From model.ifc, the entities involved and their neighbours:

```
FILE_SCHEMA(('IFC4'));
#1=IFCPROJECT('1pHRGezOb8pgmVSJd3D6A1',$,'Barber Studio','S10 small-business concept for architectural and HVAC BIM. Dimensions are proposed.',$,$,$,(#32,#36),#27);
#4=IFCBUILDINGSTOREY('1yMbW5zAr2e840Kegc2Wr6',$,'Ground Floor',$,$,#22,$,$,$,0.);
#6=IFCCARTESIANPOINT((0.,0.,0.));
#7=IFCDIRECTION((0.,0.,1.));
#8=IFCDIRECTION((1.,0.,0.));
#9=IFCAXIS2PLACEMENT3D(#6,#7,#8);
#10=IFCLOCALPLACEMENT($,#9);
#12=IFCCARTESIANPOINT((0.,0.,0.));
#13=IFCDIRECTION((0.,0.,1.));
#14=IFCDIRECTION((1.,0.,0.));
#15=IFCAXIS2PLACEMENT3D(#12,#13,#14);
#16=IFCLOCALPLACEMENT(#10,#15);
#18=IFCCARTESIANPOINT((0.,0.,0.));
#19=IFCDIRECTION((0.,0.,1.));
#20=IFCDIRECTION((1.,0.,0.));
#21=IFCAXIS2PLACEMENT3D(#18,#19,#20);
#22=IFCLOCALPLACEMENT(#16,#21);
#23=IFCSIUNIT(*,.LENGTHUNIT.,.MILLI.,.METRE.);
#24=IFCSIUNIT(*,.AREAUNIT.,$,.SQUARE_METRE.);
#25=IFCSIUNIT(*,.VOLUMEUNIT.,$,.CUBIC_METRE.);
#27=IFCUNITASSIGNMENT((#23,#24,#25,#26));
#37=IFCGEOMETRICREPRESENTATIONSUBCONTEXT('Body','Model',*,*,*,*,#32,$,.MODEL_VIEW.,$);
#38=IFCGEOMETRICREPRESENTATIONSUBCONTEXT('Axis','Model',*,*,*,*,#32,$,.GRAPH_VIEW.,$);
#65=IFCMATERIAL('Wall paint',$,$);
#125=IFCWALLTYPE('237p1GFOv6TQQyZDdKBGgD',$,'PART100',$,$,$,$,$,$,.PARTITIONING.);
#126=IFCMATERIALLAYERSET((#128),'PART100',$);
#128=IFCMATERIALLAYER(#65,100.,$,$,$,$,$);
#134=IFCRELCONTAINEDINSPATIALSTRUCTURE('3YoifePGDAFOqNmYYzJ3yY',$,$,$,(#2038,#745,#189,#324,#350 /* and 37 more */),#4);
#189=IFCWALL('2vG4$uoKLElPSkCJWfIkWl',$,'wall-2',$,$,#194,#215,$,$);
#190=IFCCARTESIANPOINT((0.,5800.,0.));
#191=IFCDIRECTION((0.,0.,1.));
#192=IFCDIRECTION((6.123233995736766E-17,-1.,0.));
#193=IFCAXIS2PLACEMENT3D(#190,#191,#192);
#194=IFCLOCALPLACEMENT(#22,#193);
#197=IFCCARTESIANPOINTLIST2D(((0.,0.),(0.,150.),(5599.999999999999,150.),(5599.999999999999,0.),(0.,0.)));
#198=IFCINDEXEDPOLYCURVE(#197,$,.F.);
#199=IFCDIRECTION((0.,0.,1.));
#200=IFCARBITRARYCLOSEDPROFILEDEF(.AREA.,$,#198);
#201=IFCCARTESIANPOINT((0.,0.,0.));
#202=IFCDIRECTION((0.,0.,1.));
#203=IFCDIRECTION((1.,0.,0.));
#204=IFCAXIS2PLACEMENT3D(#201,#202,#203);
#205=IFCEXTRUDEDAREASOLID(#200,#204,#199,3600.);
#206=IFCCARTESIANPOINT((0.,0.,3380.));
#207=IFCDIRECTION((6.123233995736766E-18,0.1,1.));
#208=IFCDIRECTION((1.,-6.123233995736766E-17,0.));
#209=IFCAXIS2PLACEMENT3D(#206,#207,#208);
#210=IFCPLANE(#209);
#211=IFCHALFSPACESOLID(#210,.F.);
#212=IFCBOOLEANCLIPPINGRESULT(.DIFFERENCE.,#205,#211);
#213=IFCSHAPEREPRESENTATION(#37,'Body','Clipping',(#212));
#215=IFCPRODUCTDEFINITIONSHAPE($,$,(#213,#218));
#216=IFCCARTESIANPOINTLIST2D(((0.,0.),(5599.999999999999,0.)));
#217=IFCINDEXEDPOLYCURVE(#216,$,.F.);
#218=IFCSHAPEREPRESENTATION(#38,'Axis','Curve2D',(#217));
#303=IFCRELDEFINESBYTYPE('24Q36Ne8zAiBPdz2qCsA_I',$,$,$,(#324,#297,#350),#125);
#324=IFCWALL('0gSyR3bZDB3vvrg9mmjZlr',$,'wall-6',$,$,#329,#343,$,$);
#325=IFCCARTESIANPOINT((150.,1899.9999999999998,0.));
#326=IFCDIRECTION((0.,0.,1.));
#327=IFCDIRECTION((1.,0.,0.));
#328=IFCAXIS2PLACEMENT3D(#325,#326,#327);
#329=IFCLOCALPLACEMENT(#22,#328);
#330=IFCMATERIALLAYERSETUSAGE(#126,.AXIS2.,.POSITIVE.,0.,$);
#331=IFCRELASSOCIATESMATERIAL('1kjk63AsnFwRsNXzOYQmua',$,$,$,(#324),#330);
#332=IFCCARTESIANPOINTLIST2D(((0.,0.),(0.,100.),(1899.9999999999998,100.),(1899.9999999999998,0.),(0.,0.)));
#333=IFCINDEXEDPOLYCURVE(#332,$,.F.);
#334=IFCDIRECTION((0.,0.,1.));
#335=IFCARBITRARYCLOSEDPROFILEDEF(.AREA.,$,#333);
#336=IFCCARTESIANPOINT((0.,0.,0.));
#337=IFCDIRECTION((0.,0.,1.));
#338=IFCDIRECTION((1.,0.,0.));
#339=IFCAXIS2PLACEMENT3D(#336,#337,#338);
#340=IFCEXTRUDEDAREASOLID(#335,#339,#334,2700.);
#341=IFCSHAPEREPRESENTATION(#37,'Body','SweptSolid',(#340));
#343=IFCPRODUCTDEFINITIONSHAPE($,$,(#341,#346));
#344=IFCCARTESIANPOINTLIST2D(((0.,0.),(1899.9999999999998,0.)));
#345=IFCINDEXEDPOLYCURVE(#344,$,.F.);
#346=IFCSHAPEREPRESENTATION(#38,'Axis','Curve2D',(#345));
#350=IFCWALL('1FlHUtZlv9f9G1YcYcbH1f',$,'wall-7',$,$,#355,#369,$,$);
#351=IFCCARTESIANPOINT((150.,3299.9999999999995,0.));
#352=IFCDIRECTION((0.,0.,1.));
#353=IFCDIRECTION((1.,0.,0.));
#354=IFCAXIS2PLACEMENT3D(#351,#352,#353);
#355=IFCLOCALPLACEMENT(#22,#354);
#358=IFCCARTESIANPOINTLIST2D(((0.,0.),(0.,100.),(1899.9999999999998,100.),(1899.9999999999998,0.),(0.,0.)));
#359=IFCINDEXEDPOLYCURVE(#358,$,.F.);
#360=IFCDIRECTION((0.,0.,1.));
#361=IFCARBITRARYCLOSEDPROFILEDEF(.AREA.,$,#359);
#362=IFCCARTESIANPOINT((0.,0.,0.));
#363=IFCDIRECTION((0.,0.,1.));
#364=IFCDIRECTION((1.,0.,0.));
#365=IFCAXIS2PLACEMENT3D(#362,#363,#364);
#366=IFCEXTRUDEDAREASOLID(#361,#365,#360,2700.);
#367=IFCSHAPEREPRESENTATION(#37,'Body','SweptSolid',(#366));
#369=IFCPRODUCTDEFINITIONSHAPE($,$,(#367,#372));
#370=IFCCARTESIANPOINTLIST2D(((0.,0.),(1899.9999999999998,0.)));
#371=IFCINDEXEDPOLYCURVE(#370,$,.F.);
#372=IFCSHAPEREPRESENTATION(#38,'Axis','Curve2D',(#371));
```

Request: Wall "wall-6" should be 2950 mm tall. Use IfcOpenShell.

```python
import ifcopenshell
import ifcopenshell.geom
import ifcopenshell.util.representation
import ifcopenshell.util.shape

model = ifcopenshell.open("model.ifc")
settings = ifcopenshell.geom.settings()


def volume(element):
    """Net volume in cubic metres, openings subtracted."""
    shape = ifcopenshell.geom.create_shape(settings, element)
    return ifcopenshell.util.shape.get_volume(shape.geometry)


wall = model.by_id(324)
before = volume(wall)

body = ifcopenshell.util.representation.get_representation(wall, "Model", "Body")
solid = body.Items[0]
old_height = solid.Depth
solid.Depth = 2950.0
after = volume(wall)

print(f"height {old_height:g} -> {solid.Depth:g}, volume {before:.3f} -> {after:.3f} m3")

model.write("model_updated.ifc")
```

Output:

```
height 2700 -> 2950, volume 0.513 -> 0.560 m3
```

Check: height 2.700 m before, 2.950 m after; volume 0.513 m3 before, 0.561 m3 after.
